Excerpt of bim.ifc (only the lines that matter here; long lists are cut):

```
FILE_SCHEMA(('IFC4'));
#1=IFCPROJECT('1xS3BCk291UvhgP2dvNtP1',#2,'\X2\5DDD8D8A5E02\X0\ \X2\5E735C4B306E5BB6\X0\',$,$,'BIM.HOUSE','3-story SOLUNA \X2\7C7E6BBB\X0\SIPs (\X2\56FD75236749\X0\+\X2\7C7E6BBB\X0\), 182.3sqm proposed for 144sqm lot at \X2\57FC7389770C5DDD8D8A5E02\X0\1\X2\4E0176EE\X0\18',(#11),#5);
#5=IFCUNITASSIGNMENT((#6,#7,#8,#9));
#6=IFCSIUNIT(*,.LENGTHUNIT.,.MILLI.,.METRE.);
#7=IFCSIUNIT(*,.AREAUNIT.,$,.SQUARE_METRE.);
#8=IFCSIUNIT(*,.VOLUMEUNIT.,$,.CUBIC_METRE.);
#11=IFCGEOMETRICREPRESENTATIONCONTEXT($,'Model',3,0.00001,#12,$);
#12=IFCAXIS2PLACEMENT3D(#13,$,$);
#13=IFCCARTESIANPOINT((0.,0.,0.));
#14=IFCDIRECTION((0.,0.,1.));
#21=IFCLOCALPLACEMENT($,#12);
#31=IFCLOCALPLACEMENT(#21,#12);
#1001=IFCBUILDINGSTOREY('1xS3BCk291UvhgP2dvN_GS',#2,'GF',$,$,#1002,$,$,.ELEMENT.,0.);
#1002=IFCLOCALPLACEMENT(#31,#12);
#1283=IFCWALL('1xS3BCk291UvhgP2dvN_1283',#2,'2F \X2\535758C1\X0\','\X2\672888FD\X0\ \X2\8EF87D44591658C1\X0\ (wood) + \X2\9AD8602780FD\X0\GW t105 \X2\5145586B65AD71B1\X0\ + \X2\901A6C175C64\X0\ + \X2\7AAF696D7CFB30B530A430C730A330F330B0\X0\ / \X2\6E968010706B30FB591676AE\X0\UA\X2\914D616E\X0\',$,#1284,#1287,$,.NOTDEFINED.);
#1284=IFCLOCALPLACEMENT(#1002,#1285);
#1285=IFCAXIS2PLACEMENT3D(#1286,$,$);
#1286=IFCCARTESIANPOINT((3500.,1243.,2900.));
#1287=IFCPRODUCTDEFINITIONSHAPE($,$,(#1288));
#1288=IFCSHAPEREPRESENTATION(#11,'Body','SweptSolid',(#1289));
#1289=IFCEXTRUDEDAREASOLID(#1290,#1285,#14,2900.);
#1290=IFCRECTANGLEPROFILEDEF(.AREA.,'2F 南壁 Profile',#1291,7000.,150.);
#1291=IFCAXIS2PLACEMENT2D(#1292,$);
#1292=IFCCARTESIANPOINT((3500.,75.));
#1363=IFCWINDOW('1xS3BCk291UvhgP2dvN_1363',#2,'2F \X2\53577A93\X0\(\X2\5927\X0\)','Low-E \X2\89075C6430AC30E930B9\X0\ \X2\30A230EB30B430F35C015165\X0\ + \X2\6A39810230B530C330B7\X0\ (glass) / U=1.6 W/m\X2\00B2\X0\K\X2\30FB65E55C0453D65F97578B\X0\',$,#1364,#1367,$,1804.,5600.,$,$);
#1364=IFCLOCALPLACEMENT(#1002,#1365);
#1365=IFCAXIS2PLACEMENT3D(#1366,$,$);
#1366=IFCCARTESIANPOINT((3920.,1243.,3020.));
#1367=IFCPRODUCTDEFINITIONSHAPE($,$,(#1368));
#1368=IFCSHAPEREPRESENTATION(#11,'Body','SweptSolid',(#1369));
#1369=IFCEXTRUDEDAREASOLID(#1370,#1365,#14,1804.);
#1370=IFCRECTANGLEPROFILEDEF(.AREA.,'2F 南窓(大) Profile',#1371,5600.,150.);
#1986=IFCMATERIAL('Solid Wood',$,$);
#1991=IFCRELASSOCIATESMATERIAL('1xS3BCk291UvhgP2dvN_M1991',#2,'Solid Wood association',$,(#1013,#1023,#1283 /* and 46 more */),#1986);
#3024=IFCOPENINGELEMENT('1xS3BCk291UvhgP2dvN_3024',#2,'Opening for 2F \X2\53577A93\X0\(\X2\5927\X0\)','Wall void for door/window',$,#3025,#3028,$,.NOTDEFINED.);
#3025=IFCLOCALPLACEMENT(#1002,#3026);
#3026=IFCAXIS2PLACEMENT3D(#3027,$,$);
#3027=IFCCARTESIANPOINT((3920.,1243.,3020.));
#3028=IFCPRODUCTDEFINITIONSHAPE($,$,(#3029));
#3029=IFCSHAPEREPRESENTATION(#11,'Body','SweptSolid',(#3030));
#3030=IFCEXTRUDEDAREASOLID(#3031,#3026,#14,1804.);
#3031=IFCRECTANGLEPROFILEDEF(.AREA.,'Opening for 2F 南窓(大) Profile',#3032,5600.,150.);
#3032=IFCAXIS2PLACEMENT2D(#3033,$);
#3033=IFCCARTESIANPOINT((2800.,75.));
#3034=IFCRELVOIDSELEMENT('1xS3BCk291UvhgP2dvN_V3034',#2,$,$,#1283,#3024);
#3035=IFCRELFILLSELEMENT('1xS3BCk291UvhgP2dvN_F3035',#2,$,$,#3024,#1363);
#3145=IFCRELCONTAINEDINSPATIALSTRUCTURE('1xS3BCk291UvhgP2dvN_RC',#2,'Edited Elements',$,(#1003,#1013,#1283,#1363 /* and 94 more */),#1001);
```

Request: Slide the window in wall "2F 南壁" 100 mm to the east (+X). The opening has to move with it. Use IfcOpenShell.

```python
import ifcopenshell
import ifcopenshell.api.geometry
import ifcopenshell.util.placement

model = ifcopenshell.open("bim.ifc")

window = model.by_guid("1xS3BCk291UvhgP2dvN_1363")
opening = window.FillsVoids[0].RelatingOpeningElement
wall = opening.VoidsElements[0].RelatingBuildingElement

wall_matrix = ifcopenshell.util.placement.get_local_placement(wall.ObjectPlacement)
shift = wall_matrix[:3, 0] * 100.0
before = ifcopenshell.util.placement.get_local_placement(window.ObjectPlacement)[:3, 3].copy()

# The window is not placed relative to its opening, so move both.
for product in (opening, window):
    matrix = ifcopenshell.util.placement.get_local_placement(product.ObjectPlacement)
    matrix[:3, 3] += shift
    ifcopenshell.api.geometry.edit_object_placement(model, product=product, matrix=matrix, is_si=False)

after = ifcopenshell.util.placement.get_local_placement(window.ObjectPlacement)[:3, 3]
print("window moved by", (after - before).round(3) + 0.0)

model.write("bim_v2.ifc")
```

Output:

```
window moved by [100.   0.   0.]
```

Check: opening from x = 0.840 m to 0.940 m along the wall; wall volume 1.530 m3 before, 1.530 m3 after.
